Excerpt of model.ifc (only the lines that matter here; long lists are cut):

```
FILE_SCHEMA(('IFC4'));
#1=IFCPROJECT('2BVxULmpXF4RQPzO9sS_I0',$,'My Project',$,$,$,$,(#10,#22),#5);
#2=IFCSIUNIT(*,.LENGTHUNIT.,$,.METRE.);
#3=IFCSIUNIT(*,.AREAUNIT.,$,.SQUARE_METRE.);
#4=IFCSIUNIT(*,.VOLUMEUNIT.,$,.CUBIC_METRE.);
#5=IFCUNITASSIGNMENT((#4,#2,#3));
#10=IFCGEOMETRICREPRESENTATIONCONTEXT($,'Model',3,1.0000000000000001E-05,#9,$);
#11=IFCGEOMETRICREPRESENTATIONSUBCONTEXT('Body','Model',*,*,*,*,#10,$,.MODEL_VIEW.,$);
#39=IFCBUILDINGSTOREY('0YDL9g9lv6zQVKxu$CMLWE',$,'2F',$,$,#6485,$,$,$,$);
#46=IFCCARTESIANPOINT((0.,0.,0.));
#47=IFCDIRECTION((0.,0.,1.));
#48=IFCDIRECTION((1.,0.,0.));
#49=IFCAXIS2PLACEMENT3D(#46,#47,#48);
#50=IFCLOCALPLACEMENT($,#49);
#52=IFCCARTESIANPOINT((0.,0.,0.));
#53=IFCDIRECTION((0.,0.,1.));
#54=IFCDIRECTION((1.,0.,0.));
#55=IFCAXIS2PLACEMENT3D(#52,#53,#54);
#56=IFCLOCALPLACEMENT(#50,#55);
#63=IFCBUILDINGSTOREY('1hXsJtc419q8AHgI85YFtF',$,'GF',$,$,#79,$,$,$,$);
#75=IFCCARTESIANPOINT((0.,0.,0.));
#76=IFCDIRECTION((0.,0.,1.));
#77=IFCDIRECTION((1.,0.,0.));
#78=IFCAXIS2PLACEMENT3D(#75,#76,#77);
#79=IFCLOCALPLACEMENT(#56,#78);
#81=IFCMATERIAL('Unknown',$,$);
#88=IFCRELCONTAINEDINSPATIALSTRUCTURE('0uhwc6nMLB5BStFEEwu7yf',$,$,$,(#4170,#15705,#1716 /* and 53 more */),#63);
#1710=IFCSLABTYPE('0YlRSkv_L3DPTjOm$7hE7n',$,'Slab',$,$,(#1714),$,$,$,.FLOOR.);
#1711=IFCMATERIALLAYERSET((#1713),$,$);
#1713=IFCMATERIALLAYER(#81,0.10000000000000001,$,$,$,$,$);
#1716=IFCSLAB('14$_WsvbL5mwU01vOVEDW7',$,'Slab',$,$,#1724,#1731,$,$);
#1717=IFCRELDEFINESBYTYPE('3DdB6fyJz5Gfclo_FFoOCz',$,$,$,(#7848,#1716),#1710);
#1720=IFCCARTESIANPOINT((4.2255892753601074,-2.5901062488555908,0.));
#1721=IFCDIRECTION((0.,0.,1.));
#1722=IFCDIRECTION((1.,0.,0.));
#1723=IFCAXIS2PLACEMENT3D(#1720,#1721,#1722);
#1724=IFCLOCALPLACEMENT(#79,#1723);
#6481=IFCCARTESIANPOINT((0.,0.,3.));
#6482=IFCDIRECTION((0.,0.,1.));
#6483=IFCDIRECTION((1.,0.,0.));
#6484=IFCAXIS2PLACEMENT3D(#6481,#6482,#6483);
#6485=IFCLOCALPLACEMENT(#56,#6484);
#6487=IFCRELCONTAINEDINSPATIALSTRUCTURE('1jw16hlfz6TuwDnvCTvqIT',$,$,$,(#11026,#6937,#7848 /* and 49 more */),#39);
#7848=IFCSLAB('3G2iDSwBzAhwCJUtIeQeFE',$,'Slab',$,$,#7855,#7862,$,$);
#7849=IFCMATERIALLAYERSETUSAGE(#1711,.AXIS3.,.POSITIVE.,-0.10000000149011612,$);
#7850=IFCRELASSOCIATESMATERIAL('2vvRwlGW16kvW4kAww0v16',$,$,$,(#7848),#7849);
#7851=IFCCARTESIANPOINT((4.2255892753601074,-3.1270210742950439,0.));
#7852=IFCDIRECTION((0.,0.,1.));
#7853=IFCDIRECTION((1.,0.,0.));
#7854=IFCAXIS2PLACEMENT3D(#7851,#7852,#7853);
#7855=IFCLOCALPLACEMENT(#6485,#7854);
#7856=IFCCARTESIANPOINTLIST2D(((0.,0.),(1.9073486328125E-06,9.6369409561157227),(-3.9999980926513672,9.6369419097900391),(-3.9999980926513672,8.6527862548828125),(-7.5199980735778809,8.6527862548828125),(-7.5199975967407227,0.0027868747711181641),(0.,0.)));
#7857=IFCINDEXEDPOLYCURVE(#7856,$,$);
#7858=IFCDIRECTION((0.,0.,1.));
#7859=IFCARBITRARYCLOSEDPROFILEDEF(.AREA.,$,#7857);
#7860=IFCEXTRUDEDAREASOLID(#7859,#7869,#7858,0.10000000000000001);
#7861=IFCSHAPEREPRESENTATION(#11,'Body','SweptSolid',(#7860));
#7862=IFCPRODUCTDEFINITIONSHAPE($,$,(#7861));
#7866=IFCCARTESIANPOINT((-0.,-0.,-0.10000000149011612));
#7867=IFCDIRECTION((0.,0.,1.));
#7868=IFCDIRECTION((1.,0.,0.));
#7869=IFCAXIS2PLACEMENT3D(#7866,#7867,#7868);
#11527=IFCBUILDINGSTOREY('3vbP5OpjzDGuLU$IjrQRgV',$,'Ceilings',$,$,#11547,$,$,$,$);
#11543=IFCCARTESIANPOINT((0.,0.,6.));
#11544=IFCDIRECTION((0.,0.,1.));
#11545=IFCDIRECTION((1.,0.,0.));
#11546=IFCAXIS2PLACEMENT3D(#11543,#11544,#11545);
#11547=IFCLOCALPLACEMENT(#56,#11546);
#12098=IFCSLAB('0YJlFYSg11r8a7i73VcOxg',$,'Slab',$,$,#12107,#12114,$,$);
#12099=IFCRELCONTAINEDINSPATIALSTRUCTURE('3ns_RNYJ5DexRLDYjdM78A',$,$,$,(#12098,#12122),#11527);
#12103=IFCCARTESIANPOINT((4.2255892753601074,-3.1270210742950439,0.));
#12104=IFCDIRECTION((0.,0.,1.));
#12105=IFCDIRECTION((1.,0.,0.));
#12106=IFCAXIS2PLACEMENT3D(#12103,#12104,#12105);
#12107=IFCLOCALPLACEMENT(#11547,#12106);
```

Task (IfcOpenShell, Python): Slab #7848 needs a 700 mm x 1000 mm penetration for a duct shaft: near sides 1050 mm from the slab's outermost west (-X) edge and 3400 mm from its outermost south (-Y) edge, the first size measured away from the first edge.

```python
import numpy as np
import ifcopenshell
import ifcopenshell.api.feature
import ifcopenshell.api.geometry
import ifcopenshell.api.root
import ifcopenshell.geom
import ifcopenshell.util.placement
import ifcopenshell.util.representation
import ifcopenshell.util.shape
import ifcopenshell.util.unit

model = ifcopenshell.open("model.ifc")
unit_scale = ifcopenshell.util.unit.calculate_unit_scale(model)
settings = ifcopenshell.geom.settings()


def volume(element):
    """Net volume in cubic metres, openings subtracted."""
    shape = ifcopenshell.geom.create_shape(settings, element)
    return ifcopenshell.util.shape.get_volume(shape.geometry)


slab = model.by_guid("3G2iDSwBzAhwCJUtIeQeFE")
before = volume(slab)

# Extent in the slab's own axes, in metres. The edges named are its -X and -Y sides.
slab_shape = ifcopenshell.geom.create_shape(settings, slab)
vertices = ifcopenshell.util.shape.get_vertices(slab_shape.geometry)
x_min, y_min, bottom = vertices.min(axis=0)
top = vertices[:, 2].max()

opening = ifcopenshell.api.root.create_entity(model, ifc_class="IfcOpeningElement", name="Duct shaft opening", predefined_type="OPENING")
context = ifcopenshell.util.representation.get_context(model, "Model", "Body", "MODEL_VIEW")
width, depth = 0.7, 1
outline = [(0.0, 0.0), (width, 0.0), (width, depth), (0.0, depth), (0.0, 0.0)]
# Overshoot both faces by 50 mm so the cut is clean.
shape = ifcopenshell.api.geometry.add_slab_representation(
    model, context=context, depth=top - bottom + 0.1, polyline=outline
)
ifcopenshell.api.geometry.assign_representation(model, product=opening, representation=shape)

matrix = ifcopenshell.util.placement.get_local_placement(slab.ObjectPlacement)
matrix[:, 3] = matrix @ np.append(np.array([x_min + 1.05, y_min + 3.4, bottom - 0.05]) / unit_scale, 1.0)
ifcopenshell.api.geometry.edit_object_placement(model, product=opening, matrix=matrix, is_si=False)
ifcopenshell.api.feature.add_feature(model, feature=opening, element=slab)

after = volume(slab)

print(f"slab volume {before:.3f} -> {after:.3f} m3")

model.write("model-out.ifc")
```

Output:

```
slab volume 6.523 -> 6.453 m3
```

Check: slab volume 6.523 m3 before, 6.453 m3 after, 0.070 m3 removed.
